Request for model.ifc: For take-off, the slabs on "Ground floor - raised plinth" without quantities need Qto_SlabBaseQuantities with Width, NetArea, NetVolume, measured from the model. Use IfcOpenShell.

First a look at what the model holds.

```python
import ifcopenshell
import ifcopenshell.util.element
import ifcopenshell.util.unit

model = ifcopenshell.open("model.ifc")
print(model.schema)
for unit_type in ("LENGTHUNIT", "AREAUNIT", "VOLUMEUNIT"):
    print(unit_type, ifcopenshell.util.unit.calculate_unit_scale(model, unit_type))
storey = next(s for s in model.by_type("IfcBuildingStorey") if s.Name == "Ground floor - raised plinth")
slabs = [e for e in ifcopenshell.util.element.get_decomposition(storey) if e.is_a("IfcSlab")]
for e in sorted(slabs, key=lambda e: e.id()):
    print(e.id(), e.is_a(), e.Name, list(ifcopenshell.util.element.get_psets(e, qtos_only=True)), sep=" | ")
```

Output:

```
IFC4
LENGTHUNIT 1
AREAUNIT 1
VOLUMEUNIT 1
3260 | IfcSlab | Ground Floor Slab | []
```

```python
import ifcopenshell
import ifcopenshell.api.pset
import ifcopenshell.geom
import ifcopenshell.util.element
import ifcopenshell.util.shape
import ifcopenshell.util.unit

model = ifcopenshell.open("model.ifc")
unit_scale = ifcopenshell.util.unit.calculate_unit_scale(model)
area_scale = ifcopenshell.util.unit.calculate_unit_scale(model, "AREAUNIT")
volume_scale = ifcopenshell.util.unit.calculate_unit_scale(model, "VOLUMEUNIT")
settings = ifcopenshell.geom.settings()

storey = next(s for s in model.by_type("IfcBuildingStorey") if s.Name == "Ground floor - raised plinth")
slabs = [e for e in ifcopenshell.util.element.get_decomposition(storey) if e.is_a("IfcSlab")]

for e in sorted(slabs, key=lambda e: e.id()):
    if ifcopenshell.util.element.get_psets(e, qtos_only=True, should_inherit=False):
        continue
    # Geometry comes back in metres, in the element's own axes.
    shape = ifcopenshell.geom.create_shape(settings, e)
    values = {
        "Width": ifcopenshell.util.shape.get_z(shape.geometry) / unit_scale,
        "NetArea": ifcopenshell.util.shape.get_footprint_area(shape.geometry) / area_scale,
        "NetVolume": ifcopenshell.util.shape.get_volume(shape.geometry) / volume_scale,
    }
    qto = ifcopenshell.api.pset.add_qto(model, product=e, name="Qto_SlabBaseQuantities")
    ifcopenshell.api.pset.edit_qto(model, qto=qto, properties=values)
    print(e.id(), {k: round(v, 3) for k, v in values.items()})

model.write("model_updated.ifc")
```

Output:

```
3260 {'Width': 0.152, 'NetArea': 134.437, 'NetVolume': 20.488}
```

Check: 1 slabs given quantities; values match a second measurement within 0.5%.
